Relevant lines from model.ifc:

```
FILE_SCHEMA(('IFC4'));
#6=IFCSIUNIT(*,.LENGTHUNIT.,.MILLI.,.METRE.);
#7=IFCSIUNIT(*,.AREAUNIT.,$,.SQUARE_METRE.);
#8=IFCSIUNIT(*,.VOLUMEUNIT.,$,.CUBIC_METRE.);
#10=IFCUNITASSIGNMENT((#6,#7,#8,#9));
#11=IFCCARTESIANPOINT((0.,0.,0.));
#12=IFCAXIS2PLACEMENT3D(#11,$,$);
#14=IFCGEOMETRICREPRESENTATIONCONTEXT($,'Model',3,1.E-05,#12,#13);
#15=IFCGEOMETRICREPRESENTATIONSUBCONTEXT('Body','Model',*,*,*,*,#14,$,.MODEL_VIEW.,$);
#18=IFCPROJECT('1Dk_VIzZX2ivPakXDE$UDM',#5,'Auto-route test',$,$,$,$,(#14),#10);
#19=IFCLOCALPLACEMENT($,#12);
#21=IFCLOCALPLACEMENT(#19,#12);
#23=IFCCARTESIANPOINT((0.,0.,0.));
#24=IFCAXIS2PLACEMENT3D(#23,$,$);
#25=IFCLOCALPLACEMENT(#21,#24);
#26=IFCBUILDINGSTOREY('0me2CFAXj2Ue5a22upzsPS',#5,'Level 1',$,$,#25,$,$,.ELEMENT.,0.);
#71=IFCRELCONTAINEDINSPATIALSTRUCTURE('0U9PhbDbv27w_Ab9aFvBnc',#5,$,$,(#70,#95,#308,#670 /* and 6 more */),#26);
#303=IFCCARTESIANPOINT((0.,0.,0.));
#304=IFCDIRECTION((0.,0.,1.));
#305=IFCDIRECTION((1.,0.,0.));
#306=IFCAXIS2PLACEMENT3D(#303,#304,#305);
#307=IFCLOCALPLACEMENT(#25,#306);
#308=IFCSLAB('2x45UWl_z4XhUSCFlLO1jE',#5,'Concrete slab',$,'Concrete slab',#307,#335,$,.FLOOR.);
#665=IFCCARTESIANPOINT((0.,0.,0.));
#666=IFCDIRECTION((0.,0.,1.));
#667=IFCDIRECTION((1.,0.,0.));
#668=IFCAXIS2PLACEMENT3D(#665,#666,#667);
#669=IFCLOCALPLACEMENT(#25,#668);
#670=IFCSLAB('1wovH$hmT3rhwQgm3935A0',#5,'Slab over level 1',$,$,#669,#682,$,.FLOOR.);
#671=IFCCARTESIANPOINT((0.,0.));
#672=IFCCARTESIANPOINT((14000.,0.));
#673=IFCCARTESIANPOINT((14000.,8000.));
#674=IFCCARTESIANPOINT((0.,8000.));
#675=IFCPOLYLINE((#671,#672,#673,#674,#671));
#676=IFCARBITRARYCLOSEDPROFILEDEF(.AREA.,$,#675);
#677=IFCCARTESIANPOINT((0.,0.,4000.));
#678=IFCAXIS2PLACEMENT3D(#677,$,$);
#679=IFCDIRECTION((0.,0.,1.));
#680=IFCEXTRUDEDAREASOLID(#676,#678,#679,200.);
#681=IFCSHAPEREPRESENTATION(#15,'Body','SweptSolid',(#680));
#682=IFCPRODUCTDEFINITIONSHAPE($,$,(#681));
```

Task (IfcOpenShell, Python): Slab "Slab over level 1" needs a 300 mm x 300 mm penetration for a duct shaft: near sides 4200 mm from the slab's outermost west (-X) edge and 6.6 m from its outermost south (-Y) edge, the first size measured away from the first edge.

```python
import numpy as np
import ifcopenshell
import ifcopenshell.api.feature
import ifcopenshell.api.geometry
import ifcopenshell.api.root
import ifcopenshell.geom
import ifcopenshell.util.placement
import ifcopenshell.util.representation
import ifcopenshell.util.shape
import ifcopenshell.util.unit

model = ifcopenshell.open("model.ifc")
unit_scale = ifcopenshell.util.unit.calculate_unit_scale(model)
settings = ifcopenshell.geom.settings()


def volume(element):
    """Net volume in cubic metres, openings subtracted."""
    shape = ifcopenshell.geom.create_shape(settings, element)
    return ifcopenshell.util.shape.get_volume(shape.geometry)


slab = model.by_id(670)
before = volume(slab)

# Extent in the slab's own axes, in metres. The edges named are its -X and -Y sides.
slab_shape = ifcopenshell.geom.create_shape(settings, slab)
vertices = ifcopenshell.util.shape.get_vertices(slab_shape.geometry)
x_min, y_min, bottom = vertices.min(axis=0)
top = vertices[:, 2].max()

opening = ifcopenshell.api.root.create_entity(model, ifc_class="IfcOpeningElement", name="Duct shaft opening", predefined_type="OPENING")
context = ifcopenshell.util.representation.get_context(model, "Model", "Body", "MODEL_VIEW")
width, depth = 0.3, 0.3
outline = [(0.0, 0.0), (width, 0.0), (width, depth), (0.0, depth), (0.0, 0.0)]
# Overshoot both faces by 50 mm so the cut is clean.
shape = ifcopenshell.api.geometry.add_slab_representation(
    model, context=context, depth=top - bottom + 0.1, polyline=outline
)
ifcopenshell.api.geometry.assign_representation(model, product=opening, representation=shape)

matrix = ifcopenshell.util.placement.get_local_placement(slab.ObjectPlacement)
matrix[:, 3] = matrix @ np.append(np.array([x_min + 4.2, y_min + 6.6, bottom - 0.05]) / unit_scale, 1.0)
ifcopenshell.api.geometry.edit_object_placement(model, product=opening, matrix=matrix, is_si=False)
ifcopenshell.api.feature.add_feature(model, feature=opening, element=slab)

after = volume(slab)

print(f"slab volume {before:.3f} -> {after:.3f} m3")

model.write("model_updated.ifc")
```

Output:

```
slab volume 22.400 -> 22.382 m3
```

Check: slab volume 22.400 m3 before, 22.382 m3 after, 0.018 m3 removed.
